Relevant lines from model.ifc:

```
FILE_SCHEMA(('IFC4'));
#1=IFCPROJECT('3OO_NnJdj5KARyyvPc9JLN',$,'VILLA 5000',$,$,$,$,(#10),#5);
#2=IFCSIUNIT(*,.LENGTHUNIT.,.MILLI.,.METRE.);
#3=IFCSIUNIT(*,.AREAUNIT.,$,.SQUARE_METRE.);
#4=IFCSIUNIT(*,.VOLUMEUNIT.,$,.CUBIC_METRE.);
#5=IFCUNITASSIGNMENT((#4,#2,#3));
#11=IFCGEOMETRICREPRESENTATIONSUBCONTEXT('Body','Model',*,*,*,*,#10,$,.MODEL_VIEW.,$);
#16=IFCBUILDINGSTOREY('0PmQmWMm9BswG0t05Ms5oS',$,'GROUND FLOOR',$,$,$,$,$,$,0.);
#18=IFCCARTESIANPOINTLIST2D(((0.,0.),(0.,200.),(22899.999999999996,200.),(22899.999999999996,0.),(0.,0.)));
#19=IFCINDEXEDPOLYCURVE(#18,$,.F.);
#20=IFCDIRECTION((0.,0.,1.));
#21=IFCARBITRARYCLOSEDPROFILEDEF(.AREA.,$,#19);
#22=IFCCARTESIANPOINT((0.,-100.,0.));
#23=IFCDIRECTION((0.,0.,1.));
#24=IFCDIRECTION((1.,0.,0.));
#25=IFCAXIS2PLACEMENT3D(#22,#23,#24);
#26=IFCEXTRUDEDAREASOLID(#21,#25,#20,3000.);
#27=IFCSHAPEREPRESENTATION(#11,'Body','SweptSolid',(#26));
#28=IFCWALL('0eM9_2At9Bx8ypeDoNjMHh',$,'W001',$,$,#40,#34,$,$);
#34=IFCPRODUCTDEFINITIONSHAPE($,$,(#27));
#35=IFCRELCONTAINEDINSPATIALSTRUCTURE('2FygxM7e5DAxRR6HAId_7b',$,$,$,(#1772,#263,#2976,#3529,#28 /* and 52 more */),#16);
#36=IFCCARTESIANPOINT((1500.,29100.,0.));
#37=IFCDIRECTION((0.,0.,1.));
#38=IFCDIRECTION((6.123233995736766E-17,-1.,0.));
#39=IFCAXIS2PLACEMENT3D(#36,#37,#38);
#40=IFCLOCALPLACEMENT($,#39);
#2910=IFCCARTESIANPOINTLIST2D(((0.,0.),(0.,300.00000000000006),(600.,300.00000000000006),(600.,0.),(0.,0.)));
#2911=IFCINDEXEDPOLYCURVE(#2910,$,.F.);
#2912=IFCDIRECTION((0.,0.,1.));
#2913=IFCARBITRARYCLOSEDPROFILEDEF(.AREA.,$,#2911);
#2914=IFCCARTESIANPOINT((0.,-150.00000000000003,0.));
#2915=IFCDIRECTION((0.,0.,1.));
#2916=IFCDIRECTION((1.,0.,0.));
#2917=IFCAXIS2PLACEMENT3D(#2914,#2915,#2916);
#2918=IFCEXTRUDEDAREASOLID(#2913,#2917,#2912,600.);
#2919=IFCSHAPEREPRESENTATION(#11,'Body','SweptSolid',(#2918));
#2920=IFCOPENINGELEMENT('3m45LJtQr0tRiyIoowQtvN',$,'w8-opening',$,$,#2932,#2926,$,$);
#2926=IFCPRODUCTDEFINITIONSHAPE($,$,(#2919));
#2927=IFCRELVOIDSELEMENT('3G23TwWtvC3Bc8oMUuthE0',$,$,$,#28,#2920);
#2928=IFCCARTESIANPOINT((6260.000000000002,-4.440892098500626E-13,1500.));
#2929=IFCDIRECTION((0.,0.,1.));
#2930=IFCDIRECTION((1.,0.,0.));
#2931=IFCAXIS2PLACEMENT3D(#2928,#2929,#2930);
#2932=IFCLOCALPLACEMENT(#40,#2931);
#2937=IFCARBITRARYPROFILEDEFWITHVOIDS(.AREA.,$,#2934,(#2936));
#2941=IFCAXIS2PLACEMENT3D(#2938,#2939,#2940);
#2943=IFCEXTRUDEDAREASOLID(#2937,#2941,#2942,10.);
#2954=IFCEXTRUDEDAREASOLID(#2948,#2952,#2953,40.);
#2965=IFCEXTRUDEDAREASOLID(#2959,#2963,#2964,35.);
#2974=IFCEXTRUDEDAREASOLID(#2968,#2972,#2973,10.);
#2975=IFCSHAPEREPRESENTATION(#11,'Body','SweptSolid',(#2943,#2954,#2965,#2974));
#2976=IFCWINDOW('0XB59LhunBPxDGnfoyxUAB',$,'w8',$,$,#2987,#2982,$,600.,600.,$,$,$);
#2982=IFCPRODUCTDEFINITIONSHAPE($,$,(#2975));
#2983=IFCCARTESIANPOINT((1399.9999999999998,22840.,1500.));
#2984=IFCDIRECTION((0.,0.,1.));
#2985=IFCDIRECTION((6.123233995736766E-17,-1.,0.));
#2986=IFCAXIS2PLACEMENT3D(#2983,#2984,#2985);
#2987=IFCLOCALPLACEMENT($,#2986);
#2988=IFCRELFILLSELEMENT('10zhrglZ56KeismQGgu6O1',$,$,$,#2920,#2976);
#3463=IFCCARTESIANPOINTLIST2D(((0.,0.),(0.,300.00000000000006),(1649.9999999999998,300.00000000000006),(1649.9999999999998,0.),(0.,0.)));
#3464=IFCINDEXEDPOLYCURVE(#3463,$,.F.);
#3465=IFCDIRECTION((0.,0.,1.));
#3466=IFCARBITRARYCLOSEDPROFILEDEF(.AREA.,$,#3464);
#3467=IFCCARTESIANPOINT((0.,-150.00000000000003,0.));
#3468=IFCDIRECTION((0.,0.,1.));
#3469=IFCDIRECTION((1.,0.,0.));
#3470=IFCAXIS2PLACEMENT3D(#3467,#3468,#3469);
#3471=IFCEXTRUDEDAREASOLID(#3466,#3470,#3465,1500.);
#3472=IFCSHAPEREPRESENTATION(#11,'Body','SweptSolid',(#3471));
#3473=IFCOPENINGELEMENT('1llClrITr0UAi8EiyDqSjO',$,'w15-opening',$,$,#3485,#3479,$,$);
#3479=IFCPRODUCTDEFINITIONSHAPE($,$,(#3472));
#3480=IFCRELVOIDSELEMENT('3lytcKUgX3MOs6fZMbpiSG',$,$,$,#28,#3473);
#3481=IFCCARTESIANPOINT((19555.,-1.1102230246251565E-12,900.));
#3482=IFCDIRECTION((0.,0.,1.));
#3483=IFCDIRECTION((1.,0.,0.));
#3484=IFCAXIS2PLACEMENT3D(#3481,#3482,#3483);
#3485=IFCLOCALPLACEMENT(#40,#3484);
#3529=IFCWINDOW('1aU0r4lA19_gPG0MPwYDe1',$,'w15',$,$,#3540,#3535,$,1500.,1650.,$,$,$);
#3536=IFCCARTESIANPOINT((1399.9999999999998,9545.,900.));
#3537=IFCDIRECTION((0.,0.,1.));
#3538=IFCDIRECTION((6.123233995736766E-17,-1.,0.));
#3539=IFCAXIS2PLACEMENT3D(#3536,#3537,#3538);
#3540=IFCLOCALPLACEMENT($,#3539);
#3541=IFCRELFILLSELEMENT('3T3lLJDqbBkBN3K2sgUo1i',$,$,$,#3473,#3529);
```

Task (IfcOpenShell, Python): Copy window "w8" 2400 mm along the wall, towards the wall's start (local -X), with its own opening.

```python
import ifcopenshell
import ifcopenshell.api.feature
import ifcopenshell.api.geometry
import ifcopenshell.api.root
import ifcopenshell.geom
import ifcopenshell.util.element
import ifcopenshell.util.placement
import ifcopenshell.util.shape

model = ifcopenshell.open("model.ifc")
settings = ifcopenshell.geom.settings()


def volume(element):
    """Net volume in cubic metres, openings subtracted."""
    shape = ifcopenshell.geom.create_shape(settings, element)
    return ifcopenshell.util.shape.get_volume(shape.geometry)


window = model.by_id(2976)
opening = window.FillsVoids[0].RelatingOpeningElement
wall = opening.VoidsElements[0].RelatingBuildingElement
before = volume(wall)
shift = ifcopenshell.util.placement.get_local_placement(wall.ObjectPlacement)[:3, 0] * -2400.0

# copy_class copies the void relationship, type, container and properties, but no geometry.
new_opening = ifcopenshell.api.root.copy_class(model, product=opening)
new_opening.Representation = ifcopenshell.util.element.copy_deep(
    model, opening.Representation, exclude=["IfcGeometricRepresentationContext", "IfcRepresentationMap"]
)
new_window = ifcopenshell.api.root.copy_class(model, product=window)
new_window.Representation = ifcopenshell.util.element.copy_deep(
    model, window.Representation, exclude=["IfcGeometricRepresentationContext", "IfcRepresentationMap"]
)
ifcopenshell.api.feature.add_filling(model, opening=new_opening, element=new_window)

for old, new in ((opening, new_opening), (window, new_window)):
    matrix = ifcopenshell.util.placement.get_local_placement(old.ObjectPlacement)
    matrix[:3, 3] += shift
    ifcopenshell.api.geometry.edit_object_placement(model, product=new, matrix=matrix, is_si=False)

after = volume(wall)

print(f"wall volume {before:.3f} -> {after:.3f} m3")

model.write("model_v2.ifc")
```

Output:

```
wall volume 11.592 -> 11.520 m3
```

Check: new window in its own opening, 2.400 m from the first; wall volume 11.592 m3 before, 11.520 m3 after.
